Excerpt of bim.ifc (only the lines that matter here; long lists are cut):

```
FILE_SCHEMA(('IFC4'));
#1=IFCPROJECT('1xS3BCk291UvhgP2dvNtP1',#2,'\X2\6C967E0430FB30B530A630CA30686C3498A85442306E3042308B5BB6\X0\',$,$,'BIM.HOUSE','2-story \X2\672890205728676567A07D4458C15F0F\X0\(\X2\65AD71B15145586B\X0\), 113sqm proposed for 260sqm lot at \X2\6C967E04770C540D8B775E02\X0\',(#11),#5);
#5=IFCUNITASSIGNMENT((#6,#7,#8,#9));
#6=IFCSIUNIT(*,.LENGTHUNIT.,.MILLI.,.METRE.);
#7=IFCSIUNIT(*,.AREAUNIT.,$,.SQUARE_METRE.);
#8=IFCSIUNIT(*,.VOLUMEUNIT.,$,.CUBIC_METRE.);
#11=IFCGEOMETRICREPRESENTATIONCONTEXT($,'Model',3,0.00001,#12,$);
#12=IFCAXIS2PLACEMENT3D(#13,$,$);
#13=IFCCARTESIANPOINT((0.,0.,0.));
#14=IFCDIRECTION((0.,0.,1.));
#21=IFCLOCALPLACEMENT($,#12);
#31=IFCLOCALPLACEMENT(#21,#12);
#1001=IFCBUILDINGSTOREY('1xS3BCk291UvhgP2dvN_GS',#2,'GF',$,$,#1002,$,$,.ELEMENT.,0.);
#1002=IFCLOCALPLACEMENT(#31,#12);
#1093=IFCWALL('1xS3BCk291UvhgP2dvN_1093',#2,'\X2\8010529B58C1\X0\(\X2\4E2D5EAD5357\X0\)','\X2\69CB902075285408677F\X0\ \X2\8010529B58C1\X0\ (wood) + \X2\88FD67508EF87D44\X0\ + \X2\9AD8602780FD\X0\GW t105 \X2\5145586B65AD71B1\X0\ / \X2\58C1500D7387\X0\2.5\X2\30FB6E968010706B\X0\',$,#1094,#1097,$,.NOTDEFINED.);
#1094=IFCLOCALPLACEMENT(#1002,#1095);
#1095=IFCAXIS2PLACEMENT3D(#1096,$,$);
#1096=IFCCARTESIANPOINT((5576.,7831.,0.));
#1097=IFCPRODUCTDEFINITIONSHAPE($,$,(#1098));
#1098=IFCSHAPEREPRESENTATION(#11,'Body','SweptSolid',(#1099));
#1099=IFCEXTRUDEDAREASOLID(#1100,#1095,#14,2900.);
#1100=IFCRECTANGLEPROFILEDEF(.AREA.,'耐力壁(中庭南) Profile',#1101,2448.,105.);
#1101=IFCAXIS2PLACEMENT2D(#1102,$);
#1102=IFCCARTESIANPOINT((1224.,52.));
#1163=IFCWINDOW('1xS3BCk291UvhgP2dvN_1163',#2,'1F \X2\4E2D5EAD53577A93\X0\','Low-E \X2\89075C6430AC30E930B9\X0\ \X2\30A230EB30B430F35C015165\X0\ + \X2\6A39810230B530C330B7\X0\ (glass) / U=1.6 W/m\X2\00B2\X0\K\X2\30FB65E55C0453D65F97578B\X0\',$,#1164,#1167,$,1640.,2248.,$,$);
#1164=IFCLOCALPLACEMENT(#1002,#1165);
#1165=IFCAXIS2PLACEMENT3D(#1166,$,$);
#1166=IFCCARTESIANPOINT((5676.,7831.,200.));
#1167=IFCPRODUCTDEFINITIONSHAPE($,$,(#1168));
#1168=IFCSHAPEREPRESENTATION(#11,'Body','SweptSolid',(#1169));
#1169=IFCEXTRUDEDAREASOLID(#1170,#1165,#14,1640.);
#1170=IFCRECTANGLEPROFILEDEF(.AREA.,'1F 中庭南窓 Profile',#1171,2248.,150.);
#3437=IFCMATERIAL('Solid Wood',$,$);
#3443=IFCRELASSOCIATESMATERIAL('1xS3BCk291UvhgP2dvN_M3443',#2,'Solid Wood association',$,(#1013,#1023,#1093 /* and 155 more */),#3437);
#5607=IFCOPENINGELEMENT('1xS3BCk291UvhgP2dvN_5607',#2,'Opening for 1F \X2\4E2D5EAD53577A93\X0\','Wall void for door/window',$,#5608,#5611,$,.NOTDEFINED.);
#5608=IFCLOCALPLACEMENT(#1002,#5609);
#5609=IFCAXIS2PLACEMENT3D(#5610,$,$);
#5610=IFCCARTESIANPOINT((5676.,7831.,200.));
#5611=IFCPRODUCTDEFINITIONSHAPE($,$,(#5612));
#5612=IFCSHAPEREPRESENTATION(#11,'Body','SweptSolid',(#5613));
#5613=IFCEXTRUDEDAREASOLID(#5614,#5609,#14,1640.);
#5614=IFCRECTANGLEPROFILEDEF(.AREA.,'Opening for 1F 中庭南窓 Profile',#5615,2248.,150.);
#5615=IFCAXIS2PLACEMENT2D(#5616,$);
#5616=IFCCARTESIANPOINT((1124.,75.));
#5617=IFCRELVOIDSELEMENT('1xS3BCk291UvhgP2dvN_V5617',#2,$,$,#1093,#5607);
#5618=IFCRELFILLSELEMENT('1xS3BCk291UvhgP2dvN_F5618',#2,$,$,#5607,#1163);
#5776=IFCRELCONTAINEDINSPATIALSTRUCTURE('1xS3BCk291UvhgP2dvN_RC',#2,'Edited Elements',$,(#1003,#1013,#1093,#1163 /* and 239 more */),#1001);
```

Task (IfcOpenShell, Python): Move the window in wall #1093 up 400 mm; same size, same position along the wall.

```python
import numpy as np
import ifcopenshell
import ifcopenshell.api.geometry
import ifcopenshell.util.placement
import ifcopenshell.util.unit

model = ifcopenshell.open("bim.ifc")
unit_scale = ifcopenshell.util.unit.calculate_unit_scale(model)

window = model.by_guid("1xS3BCk291UvhgP2dvN_1163")
opening = window.FillsVoids[0].RelatingOpeningElement
dz = 0.4 / unit_scale

shift = np.array([0.0, 0.0, dz])
# The window is not placed relative to its opening, so move both.
for product in (opening, window):
    matrix = ifcopenshell.util.placement.get_local_placement(product.ObjectPlacement)
    matrix[:3, 3] += shift
    ifcopenshell.api.geometry.edit_object_placement(model, product=product, matrix=matrix, is_si=False)

print(f"moved by {dz * unit_scale:+.3f} m")

model.write("bim_rev.ifc")
```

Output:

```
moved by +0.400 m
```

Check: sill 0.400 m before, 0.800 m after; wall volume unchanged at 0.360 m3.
